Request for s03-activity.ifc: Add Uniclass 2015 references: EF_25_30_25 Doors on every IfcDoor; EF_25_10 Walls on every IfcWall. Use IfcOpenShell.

First a look at what the model holds.

```python
import ifcopenshell

model = ifcopenshell.open("s03-activity.ifc")
print(model.schema)
print("classifications:", [c.Name for c in model.by_type("IfcClassification")])
for ifc_class in ("IfcDoor", "IfcRoof", "IfcStair", "IfcWall", "IfcWindow"):
    print(ifc_class, len(model.by_type(ifc_class)))
```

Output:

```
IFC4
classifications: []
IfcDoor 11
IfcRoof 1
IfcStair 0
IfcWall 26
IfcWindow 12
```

```python
import ifcopenshell
import ifcopenshell.api.classification

model = ifcopenshell.open("s03-activity.ifc")

system = ifcopenshell.api.classification.add_classification(model, classification="Uniclass 2015")

codes = {
    "IfcDoor": ("EF_25_30_25", "Doors"),
    "IfcWall": ("EF_25_10", "Walls"),
}
for ifc_class, (code, name) in codes.items():
    products = model.by_type(ifc_class)
    ifcopenshell.api.classification.add_reference(
        model, products=products, classification=system, identification=code, name=name
    )
    print(code, len(products))

model.write("s03-activity_v2.ifc")
```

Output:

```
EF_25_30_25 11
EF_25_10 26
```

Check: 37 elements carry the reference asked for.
